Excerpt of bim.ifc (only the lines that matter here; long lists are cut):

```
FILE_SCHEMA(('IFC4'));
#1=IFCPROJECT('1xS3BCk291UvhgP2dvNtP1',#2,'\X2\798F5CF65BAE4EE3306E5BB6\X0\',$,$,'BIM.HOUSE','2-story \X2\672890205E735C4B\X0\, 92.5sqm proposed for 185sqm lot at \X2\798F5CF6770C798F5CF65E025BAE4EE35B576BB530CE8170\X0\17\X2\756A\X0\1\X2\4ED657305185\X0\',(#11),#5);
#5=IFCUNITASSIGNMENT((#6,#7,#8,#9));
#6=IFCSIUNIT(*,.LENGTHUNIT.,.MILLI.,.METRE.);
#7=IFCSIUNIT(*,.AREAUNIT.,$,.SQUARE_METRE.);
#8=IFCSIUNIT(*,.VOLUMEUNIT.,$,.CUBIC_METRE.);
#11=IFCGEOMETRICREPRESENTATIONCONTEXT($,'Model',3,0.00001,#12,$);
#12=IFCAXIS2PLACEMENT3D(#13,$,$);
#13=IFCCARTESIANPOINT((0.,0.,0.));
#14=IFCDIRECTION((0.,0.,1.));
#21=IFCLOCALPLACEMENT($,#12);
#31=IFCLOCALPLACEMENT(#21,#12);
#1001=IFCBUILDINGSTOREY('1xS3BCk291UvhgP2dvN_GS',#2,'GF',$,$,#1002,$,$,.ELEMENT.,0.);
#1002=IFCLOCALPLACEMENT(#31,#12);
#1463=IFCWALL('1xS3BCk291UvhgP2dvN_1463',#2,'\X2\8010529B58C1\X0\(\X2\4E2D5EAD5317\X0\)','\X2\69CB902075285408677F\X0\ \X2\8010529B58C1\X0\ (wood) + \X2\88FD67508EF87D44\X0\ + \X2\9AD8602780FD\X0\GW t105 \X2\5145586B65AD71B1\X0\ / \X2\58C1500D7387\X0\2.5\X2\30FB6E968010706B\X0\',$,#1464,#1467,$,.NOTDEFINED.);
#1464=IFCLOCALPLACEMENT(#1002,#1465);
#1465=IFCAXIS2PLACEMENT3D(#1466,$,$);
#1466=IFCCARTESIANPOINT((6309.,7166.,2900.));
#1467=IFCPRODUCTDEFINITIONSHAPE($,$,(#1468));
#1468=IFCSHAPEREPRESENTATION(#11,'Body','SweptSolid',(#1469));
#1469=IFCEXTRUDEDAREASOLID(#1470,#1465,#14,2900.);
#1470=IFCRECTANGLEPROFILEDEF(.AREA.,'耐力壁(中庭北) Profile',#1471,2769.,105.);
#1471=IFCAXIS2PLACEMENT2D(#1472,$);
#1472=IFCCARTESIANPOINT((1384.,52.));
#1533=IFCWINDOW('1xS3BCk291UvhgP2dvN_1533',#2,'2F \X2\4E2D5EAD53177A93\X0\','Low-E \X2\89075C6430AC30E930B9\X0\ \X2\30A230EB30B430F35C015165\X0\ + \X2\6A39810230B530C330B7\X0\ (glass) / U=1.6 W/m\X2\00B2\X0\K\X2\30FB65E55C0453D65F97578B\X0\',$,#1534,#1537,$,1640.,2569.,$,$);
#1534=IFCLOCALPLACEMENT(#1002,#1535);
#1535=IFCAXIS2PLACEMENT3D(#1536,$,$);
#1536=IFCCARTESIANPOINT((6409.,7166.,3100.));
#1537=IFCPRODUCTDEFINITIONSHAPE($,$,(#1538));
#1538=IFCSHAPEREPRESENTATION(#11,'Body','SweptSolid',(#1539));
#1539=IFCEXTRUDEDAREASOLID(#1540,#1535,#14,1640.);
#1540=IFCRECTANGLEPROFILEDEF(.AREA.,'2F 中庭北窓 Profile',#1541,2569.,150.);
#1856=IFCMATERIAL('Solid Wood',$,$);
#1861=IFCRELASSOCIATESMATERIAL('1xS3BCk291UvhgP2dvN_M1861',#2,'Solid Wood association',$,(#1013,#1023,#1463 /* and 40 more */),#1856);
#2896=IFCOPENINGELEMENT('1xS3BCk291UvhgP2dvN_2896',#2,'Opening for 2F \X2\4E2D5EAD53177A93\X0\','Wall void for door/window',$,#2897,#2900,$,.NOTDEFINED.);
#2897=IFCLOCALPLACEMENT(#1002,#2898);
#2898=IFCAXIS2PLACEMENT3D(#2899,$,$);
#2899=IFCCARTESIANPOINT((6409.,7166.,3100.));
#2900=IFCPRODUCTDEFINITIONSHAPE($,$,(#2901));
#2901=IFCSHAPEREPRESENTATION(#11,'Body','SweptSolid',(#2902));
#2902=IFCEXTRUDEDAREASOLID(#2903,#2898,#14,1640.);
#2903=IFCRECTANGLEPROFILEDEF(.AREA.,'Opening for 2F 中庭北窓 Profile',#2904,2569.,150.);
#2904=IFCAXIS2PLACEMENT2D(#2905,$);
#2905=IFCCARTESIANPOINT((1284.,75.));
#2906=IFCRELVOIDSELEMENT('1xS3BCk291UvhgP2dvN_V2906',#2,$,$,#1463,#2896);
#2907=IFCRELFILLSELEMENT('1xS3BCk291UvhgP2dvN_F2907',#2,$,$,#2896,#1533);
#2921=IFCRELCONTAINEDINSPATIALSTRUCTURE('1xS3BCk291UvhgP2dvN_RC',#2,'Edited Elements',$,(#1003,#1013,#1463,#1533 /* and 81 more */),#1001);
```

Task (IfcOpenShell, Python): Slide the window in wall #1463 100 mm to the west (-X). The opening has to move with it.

```python
import ifcopenshell
import ifcopenshell.api.geometry
import ifcopenshell.util.placement
import ifcopenshell.util.unit

model = ifcopenshell.open("bim.ifc")
unit_scale = ifcopenshell.util.unit.calculate_unit_scale(model)

window = model.by_guid("1xS3BCk291UvhgP2dvN_1533")
opening = window.FillsVoids[0].RelatingOpeningElement
wall = opening.VoidsElements[0].RelatingBuildingElement

wall_matrix = ifcopenshell.util.placement.get_local_placement(wall.ObjectPlacement)
shift = wall_matrix[:3, 0] * -0.1 / unit_scale
before = ifcopenshell.util.placement.get_local_placement(window.ObjectPlacement)[:3, 3].copy()

# The window is not placed relative to its opening, so move both.
for product in (opening, window):
    matrix = ifcopenshell.util.placement.get_local_placement(product.ObjectPlacement)
    matrix[:3, 3] += shift
    ifcopenshell.api.geometry.edit_object_placement(model, product=product, matrix=matrix, is_si=False)

after = ifcopenshell.util.placement.get_local_placement(window.ObjectPlacement)[:3, 3]
print("window moved by", (after - before).round(3) + 0.0)

model.write("bim_rev.ifc")
```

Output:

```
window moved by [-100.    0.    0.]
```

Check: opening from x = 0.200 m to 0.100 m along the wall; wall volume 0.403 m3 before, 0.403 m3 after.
